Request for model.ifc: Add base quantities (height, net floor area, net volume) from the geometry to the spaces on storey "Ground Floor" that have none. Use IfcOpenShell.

First a look at what the model holds.

```python
import ifcopenshell
import ifcopenshell.util.element
import ifcopenshell.util.unit

model = ifcopenshell.open("model.ifc")
print(model.schema)
for unit_type in ("LENGTHUNIT", "AREAUNIT", "VOLUMEUNIT"):
    print(unit_type, ifcopenshell.util.unit.calculate_unit_scale(model, unit_type))
storey = next(s for s in model.by_type("IfcBuildingStorey") if s.Name == "Ground Floor")
spaces = [e for e in ifcopenshell.util.element.get_decomposition(storey) if e.is_a("IfcSpace")]
for e in sorted(spaces, key=lambda e: e.id()):
    print(e.id(), e.is_a(), e.Name, list(ifcopenshell.util.element.get_psets(e, qtos_only=True)), sep=" | ")
```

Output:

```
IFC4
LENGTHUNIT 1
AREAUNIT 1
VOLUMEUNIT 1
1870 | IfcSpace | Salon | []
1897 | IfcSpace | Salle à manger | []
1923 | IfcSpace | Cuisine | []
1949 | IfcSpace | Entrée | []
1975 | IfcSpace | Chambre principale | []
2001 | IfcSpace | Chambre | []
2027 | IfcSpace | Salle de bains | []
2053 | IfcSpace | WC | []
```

```python
import ifcopenshell
import ifcopenshell.api.pset
import ifcopenshell.geom
import ifcopenshell.util.element
import ifcopenshell.util.shape
import ifcopenshell.util.unit

model = ifcopenshell.open("model.ifc")
unit_scale = ifcopenshell.util.unit.calculate_unit_scale(model)
area_scale = ifcopenshell.util.unit.calculate_unit_scale(model, "AREAUNIT")
volume_scale = ifcopenshell.util.unit.calculate_unit_scale(model, "VOLUMEUNIT")
settings = ifcopenshell.geom.settings()

storey = next(s for s in model.by_type("IfcBuildingStorey") if s.Name == "Ground Floor")
spaces = [e for e in ifcopenshell.util.element.get_decomposition(storey) if e.is_a("IfcSpace")]

for e in sorted(spaces, key=lambda e: e.id()):
    if ifcopenshell.util.element.get_psets(e, qtos_only=True, should_inherit=False):
        continue
    # Geometry comes back in metres, in the element's own axes.
    shape = ifcopenshell.geom.create_shape(settings, e)
    values = {
        "Height": ifcopenshell.util.shape.get_z(shape.geometry) / unit_scale,
        "NetFloorArea": ifcopenshell.util.shape.get_footprint_area(shape.geometry) / area_scale,
        "NetVolume": ifcopenshell.util.shape.get_volume(shape.geometry) / volume_scale,
    }
    qto = ifcopenshell.api.pset.add_qto(model, product=e, name="Qto_SpaceBaseQuantities")
    ifcopenshell.api.pset.edit_qto(model, qto=qto, properties=values)
    print(e.id(), {k: round(v, 3) for k, v in values.items()})

model.write("model_edited.ifc")
```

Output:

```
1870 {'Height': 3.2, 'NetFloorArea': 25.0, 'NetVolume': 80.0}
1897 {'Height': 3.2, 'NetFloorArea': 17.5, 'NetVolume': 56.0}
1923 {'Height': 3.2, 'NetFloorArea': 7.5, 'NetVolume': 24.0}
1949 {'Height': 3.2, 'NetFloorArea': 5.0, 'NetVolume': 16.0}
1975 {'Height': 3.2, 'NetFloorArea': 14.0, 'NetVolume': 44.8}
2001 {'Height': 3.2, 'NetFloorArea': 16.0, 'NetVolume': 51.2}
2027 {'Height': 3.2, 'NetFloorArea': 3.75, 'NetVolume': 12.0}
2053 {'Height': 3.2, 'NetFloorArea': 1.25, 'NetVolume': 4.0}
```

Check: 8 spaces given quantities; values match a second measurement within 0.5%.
